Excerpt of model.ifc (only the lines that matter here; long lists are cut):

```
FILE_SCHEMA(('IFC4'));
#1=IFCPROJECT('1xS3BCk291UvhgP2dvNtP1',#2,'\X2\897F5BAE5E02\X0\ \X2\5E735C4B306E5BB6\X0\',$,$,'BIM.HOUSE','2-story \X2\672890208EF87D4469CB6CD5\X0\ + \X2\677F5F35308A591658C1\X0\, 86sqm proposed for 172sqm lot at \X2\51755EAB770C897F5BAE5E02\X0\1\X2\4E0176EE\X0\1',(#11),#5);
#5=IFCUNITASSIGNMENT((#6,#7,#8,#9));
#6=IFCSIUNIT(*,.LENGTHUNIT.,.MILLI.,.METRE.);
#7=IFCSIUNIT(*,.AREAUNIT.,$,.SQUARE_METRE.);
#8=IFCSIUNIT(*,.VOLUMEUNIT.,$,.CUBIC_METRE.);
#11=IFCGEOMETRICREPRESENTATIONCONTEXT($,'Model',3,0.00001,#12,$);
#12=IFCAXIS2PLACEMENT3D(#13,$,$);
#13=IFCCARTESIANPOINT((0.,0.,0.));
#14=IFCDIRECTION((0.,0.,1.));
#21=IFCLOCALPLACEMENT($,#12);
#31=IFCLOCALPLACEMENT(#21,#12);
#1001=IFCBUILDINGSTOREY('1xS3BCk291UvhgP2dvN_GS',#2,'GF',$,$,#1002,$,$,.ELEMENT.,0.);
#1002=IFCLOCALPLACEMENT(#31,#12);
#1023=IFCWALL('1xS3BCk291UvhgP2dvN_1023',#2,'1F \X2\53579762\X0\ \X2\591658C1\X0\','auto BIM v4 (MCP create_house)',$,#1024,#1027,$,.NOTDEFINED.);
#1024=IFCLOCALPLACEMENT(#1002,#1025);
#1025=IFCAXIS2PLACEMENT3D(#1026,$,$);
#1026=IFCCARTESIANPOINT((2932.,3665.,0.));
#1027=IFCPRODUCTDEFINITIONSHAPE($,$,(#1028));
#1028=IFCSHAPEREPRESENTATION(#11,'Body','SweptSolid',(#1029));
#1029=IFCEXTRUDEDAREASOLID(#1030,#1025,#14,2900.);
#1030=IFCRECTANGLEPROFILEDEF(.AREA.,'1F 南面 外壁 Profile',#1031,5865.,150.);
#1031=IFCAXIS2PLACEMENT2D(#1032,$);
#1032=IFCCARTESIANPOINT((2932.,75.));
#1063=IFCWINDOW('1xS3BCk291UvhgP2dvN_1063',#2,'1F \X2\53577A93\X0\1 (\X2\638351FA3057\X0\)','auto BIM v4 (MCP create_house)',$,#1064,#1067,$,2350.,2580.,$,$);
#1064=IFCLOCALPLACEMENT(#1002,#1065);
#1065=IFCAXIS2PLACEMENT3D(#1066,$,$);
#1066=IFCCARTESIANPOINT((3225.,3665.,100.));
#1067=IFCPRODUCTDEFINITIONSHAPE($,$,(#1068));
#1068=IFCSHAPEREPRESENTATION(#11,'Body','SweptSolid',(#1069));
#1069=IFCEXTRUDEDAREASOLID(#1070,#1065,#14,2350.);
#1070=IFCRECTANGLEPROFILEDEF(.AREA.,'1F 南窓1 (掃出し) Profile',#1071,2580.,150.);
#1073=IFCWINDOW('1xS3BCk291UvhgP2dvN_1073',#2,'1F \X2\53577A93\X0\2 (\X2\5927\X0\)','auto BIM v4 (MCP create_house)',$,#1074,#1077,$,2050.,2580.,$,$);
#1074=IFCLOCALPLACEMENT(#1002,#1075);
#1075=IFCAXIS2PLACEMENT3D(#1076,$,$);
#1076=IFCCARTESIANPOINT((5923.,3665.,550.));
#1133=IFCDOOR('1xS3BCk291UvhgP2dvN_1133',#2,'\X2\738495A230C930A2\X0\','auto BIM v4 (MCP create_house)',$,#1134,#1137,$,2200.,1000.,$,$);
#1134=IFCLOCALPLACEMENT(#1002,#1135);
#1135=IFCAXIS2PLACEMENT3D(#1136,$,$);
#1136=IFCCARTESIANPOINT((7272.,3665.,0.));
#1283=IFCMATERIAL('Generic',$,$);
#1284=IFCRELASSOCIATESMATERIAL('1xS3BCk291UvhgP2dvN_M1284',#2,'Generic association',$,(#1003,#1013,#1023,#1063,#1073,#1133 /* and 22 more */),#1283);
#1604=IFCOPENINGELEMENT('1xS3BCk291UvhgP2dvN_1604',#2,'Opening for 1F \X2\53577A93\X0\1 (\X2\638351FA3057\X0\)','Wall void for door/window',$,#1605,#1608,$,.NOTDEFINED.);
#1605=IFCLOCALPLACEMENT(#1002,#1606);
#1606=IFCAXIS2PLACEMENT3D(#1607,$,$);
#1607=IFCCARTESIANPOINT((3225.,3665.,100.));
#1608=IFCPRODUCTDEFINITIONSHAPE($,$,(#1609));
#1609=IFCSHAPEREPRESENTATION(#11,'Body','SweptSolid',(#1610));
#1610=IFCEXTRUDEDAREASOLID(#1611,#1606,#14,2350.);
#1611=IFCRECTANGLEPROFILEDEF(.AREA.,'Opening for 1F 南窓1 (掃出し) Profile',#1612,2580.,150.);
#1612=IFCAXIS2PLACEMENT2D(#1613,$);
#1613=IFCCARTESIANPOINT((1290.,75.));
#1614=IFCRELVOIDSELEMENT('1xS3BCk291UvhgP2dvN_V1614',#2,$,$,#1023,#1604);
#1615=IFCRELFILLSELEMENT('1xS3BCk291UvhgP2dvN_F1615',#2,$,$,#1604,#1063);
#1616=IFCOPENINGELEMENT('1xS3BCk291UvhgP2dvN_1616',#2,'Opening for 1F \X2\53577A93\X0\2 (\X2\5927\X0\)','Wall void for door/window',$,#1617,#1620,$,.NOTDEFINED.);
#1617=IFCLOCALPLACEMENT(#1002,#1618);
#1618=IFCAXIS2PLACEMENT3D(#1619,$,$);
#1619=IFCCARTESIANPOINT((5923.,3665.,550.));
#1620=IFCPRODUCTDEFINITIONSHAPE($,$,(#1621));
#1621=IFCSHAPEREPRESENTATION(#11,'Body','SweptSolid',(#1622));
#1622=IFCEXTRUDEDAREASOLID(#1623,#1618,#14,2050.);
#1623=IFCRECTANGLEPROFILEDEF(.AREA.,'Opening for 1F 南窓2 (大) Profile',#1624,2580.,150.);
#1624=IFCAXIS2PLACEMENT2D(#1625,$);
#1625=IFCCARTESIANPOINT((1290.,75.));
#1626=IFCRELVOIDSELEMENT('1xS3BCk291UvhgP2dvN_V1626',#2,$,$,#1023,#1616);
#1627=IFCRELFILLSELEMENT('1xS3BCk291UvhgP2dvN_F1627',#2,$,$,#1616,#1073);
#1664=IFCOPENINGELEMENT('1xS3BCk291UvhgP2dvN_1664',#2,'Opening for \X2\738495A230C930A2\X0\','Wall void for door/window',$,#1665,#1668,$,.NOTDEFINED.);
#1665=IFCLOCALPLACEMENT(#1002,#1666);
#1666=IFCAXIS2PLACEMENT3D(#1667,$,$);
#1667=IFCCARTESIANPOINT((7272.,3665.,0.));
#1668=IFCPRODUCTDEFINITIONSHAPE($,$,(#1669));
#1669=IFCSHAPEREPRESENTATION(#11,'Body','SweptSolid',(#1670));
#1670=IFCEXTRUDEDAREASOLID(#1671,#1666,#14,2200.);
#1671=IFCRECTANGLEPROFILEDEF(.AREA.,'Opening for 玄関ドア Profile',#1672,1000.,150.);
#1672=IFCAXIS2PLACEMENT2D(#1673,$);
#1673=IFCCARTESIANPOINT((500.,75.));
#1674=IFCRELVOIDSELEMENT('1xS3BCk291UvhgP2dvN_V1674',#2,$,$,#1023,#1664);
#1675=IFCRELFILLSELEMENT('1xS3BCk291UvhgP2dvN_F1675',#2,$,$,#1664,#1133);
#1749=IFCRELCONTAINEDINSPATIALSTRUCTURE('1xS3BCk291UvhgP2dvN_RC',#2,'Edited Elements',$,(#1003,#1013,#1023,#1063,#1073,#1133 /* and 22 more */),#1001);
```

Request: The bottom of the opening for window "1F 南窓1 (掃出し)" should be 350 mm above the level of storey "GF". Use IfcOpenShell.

```python
import numpy as np
import ifcopenshell
import ifcopenshell.api.geometry
import ifcopenshell.geom
import ifcopenshell.util.element
import ifcopenshell.util.placement
import ifcopenshell.util.shape
import ifcopenshell.util.unit

model = ifcopenshell.open("model.ifc")
unit_scale = ifcopenshell.util.unit.calculate_unit_scale(model)

window = model.by_guid("1xS3BCk291UvhgP2dvN_1063")
opening = window.FillsVoids[0].RelatingOpeningElement
storey = ifcopenshell.util.element.get_container(window, ifc_class="IfcBuildingStorey")
level = ifcopenshell.util.placement.get_local_placement(storey.ObjectPlacement)[2, 3]

# The opening's origin need not be at the sill, so measure its lowest point.
shape = ifcopenshell.geom.create_shape(ifcopenshell.geom.settings(), opening)
bottom = ifcopenshell.util.shape.get_shape_bottom_elevation(shape, shape.geometry) / unit_scale
dz = level + 350.0 - bottom

shift = np.array([0.0, 0.0, dz])
# The window is not placed relative to its opening, so move both.
for product in (opening, window):
    matrix = ifcopenshell.util.placement.get_local_placement(product.ObjectPlacement)
    matrix[:3, 3] += shift
    ifcopenshell.api.geometry.edit_object_placement(model, product=product, matrix=matrix, is_si=False)

print(f"moved by {dz * unit_scale:+.3f} m")

model.write("model_rev.ifc")
```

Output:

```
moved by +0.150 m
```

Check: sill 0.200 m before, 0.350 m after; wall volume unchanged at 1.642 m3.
